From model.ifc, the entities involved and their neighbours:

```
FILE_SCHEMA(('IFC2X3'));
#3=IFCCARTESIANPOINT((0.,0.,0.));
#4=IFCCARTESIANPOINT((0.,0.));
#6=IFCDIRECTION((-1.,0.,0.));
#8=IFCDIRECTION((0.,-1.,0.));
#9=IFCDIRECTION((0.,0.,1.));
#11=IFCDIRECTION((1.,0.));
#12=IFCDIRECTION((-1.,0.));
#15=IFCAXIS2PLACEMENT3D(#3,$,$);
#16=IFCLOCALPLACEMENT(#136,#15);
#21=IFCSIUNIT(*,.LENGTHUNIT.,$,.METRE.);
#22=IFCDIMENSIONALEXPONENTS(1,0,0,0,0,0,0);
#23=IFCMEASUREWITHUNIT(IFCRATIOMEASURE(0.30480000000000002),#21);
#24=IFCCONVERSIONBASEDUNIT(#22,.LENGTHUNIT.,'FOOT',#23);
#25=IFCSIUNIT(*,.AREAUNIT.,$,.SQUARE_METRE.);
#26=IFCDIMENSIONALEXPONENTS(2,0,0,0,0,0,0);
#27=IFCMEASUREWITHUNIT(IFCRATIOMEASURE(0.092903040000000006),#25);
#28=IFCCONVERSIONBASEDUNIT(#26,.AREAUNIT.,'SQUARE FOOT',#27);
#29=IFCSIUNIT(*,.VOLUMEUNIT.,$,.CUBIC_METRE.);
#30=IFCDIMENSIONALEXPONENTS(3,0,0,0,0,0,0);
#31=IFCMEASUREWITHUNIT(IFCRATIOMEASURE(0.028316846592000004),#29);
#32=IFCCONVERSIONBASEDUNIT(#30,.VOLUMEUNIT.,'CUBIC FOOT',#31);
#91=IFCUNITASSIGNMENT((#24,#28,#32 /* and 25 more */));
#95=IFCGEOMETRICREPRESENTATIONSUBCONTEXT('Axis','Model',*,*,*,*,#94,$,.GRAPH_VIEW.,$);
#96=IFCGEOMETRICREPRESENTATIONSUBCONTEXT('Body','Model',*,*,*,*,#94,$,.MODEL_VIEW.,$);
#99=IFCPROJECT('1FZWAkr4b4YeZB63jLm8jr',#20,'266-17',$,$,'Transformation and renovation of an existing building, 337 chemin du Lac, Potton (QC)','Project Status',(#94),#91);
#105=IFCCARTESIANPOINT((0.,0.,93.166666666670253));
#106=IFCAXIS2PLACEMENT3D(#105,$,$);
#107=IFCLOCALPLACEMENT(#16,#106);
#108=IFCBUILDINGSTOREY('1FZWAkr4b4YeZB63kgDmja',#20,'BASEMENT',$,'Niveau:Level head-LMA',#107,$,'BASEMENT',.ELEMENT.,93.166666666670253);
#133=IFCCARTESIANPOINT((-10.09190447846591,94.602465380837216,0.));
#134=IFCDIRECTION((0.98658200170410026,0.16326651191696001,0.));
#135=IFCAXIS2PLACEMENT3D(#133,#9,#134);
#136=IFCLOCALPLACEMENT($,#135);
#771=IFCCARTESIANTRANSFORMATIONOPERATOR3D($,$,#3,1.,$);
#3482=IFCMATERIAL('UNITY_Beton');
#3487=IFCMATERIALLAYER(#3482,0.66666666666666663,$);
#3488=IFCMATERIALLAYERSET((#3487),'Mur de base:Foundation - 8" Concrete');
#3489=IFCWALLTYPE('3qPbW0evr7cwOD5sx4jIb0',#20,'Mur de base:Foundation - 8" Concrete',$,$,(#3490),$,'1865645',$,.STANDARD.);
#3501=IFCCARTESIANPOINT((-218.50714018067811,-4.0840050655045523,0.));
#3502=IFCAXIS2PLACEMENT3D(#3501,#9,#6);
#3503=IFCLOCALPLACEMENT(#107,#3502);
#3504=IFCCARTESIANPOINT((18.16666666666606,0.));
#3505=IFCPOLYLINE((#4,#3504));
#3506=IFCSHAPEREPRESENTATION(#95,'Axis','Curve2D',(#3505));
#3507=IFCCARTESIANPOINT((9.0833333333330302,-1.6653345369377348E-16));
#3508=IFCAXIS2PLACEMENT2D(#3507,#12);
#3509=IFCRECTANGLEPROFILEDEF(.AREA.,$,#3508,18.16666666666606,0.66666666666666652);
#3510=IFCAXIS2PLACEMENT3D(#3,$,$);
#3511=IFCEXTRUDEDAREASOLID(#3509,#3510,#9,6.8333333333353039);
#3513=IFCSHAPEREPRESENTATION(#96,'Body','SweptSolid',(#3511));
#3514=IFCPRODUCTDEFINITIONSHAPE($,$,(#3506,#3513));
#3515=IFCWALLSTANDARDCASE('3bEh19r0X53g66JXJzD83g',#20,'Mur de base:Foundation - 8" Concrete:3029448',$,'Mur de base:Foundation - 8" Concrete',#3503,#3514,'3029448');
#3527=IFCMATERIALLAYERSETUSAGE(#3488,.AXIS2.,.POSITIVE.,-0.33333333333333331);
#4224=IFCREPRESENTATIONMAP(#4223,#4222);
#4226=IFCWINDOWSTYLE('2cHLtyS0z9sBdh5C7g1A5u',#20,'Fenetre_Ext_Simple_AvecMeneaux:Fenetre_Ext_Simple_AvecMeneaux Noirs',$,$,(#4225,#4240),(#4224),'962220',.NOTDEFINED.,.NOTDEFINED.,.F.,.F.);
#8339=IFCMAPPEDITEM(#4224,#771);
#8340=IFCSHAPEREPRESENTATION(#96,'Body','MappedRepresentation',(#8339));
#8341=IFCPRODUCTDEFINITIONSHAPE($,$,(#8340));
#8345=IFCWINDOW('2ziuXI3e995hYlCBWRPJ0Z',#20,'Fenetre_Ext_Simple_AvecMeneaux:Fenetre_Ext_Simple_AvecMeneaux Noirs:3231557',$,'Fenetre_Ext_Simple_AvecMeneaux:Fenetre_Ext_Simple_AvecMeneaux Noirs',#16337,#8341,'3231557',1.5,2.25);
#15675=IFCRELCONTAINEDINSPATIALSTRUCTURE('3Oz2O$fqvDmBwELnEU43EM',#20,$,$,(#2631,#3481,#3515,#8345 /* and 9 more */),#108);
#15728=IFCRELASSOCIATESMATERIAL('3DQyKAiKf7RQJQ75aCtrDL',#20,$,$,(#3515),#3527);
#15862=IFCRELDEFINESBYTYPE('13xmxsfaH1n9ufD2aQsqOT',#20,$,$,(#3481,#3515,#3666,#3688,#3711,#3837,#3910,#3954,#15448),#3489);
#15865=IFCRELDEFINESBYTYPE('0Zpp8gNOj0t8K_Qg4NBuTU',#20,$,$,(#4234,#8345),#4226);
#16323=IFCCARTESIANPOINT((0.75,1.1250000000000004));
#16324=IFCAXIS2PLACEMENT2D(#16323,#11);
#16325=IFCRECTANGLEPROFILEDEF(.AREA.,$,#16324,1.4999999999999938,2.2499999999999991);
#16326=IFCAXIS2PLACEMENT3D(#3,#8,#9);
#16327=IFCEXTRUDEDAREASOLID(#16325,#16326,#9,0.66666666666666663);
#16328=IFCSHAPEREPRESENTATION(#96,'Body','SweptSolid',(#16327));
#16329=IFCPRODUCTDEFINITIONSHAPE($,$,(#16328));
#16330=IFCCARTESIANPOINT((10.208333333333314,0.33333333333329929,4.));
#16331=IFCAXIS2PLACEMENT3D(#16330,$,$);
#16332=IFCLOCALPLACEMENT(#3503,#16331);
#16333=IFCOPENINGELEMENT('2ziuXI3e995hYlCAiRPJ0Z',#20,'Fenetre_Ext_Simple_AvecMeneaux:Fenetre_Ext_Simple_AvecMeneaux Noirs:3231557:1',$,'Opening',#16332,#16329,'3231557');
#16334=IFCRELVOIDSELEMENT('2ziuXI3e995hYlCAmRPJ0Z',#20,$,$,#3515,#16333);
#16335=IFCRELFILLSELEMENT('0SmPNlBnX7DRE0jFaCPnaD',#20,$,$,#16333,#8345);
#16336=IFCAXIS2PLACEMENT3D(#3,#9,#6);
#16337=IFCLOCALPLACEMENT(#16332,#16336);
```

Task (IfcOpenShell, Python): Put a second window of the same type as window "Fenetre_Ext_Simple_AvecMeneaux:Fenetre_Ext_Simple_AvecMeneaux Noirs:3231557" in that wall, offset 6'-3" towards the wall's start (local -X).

```python
import ifcopenshell
import ifcopenshell.api.feature
import ifcopenshell.api.geometry
import ifcopenshell.api.root
import ifcopenshell.geom
import ifcopenshell.util.element
import ifcopenshell.util.placement
import ifcopenshell.util.shape
import ifcopenshell.util.unit

model = ifcopenshell.open("model.ifc")
unit_scale = ifcopenshell.util.unit.calculate_unit_scale(model)
settings = ifcopenshell.geom.settings()


def volume(element):
    """Net volume in cubic metres, openings subtracted."""
    shape = ifcopenshell.geom.create_shape(settings, element)
    return ifcopenshell.util.shape.get_volume(shape.geometry)


def reuse_history(source, copy):
    """copy_class also copies each property set's owner history, people and application; keep the originals."""
    for rel in copy.IsDefinedBy:
        if rel.is_a("IfcRelDefinesByProperties") and (history := rel.RelatingPropertyDefinition.OwnerHistory):
            rel.RelatingPropertyDefinition.OwnerHistory = source.OwnerHistory
            ifcopenshell.util.element.remove_deep2(model, history)


window = model.by_id(8345)
opening = window.FillsVoids[0].RelatingOpeningElement
wall = opening.VoidsElements[0].RelatingBuildingElement
before = volume(wall)
shift = ifcopenshell.util.placement.get_local_placement(wall.ObjectPlacement)[:3, 0] * -75 * 0.0254 / unit_scale

# copy_class copies the void relationship, type, container and properties, but no geometry.
new_opening = ifcopenshell.api.root.copy_class(model, product=opening)
new_opening.Representation = ifcopenshell.util.element.copy_deep(
    model, opening.Representation, exclude=["IfcGeometricRepresentationContext", "IfcRepresentationMap"]
)
new_opening.Name = "Fenetre_Ext_Simple_AvecMeneaux:Fenetre_Ext_Simple_AvecMeneaux Noirs"
new_opening.Tag = None
new_window = ifcopenshell.api.root.copy_class(model, product=window)
new_window.Representation = ifcopenshell.util.element.copy_deep(
    model, window.Representation, exclude=["IfcGeometricRepresentationContext", "IfcRepresentationMap"]
)
new_window.Name = "Fenetre_Ext_Simple_AvecMeneaux:Fenetre_Ext_Simple_AvecMeneaux Noirs"
new_window.Tag = None
reuse_history(window, new_window)
fills = ifcopenshell.api.feature.add_filling(model, opening=new_opening, element=new_window)
fills.OwnerHistory = new_window.OwnerHistory  # required in IFC2X3

for old, new in ((opening, new_opening), (window, new_window)):
    matrix = ifcopenshell.util.placement.get_local_placement(old.ObjectPlacement)
    matrix[:3, 3] += shift
    ifcopenshell.api.geometry.edit_object_placement(model, product=new, matrix=matrix, is_si=False)

after = volume(wall)

print(f"wall volume {before:.3f} -> {after:.3f} m3")

model.write("model_v2.ifc")
```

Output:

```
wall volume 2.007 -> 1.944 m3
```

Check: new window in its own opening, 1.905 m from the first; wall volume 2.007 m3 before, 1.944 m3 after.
